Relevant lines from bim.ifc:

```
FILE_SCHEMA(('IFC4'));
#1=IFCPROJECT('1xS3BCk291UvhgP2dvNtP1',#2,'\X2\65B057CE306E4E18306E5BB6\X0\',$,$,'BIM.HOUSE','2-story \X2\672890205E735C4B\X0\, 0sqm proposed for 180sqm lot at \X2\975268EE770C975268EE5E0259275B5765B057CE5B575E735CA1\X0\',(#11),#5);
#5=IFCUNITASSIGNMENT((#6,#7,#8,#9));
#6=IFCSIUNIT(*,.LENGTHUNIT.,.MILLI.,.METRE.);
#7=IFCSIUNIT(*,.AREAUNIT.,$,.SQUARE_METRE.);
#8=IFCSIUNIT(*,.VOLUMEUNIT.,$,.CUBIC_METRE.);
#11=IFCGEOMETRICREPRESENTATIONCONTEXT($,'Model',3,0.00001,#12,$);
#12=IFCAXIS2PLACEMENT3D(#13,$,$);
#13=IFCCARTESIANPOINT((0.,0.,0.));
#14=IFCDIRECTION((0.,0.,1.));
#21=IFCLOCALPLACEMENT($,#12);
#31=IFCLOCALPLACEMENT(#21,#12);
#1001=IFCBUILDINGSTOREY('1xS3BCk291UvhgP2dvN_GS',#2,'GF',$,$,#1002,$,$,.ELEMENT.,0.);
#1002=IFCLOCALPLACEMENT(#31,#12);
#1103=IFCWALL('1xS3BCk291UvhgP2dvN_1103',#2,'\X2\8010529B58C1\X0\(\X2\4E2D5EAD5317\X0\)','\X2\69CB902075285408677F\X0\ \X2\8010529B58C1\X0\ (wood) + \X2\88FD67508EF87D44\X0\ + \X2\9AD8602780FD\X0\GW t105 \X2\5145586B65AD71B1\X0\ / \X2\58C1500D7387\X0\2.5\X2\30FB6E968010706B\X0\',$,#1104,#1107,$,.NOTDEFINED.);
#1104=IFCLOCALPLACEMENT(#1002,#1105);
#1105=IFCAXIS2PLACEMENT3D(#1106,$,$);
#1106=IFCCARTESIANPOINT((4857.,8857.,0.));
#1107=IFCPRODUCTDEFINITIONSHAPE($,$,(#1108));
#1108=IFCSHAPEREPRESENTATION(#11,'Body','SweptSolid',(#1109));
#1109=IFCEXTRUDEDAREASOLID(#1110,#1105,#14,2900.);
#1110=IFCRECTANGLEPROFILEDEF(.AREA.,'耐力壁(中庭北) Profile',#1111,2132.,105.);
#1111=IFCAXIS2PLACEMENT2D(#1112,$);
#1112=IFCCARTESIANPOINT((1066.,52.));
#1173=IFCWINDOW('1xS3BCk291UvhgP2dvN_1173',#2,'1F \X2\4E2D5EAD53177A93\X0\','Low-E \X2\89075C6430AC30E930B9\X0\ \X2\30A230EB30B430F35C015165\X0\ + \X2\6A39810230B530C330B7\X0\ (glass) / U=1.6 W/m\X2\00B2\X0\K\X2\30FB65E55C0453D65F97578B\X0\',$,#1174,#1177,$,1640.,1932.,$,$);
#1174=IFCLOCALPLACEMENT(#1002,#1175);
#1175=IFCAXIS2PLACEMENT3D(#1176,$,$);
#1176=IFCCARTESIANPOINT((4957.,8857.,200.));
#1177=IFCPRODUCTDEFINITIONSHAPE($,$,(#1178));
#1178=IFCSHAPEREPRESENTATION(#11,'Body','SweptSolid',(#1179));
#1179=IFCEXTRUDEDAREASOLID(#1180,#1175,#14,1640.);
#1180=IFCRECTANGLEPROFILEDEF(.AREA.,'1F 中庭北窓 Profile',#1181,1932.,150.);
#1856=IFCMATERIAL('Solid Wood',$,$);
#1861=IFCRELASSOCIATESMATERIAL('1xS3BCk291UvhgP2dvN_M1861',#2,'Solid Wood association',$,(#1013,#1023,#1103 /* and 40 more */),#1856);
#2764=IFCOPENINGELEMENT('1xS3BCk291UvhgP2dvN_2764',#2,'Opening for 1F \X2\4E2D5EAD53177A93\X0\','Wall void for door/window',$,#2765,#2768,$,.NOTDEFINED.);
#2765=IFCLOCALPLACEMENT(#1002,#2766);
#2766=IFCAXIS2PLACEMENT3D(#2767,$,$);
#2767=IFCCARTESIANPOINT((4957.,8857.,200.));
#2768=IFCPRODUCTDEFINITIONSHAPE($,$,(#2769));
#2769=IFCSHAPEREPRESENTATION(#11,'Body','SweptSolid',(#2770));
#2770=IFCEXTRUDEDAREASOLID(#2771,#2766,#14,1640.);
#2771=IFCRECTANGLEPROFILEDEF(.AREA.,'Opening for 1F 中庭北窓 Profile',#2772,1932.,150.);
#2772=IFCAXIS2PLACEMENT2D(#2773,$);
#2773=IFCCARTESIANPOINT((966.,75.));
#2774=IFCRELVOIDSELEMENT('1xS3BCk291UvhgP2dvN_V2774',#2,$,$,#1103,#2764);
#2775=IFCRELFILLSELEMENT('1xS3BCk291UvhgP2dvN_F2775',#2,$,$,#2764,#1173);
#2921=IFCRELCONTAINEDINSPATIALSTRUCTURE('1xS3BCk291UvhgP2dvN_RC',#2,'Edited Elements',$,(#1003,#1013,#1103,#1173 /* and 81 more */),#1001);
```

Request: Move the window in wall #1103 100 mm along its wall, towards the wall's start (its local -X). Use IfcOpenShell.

```python
import ifcopenshell
import ifcopenshell.api.geometry
import ifcopenshell.util.placement

model = ifcopenshell.open("bim.ifc")

window = model.by_id(1173)
opening = window.FillsVoids[0].RelatingOpeningElement
wall = opening.VoidsElements[0].RelatingBuildingElement

wall_matrix = ifcopenshell.util.placement.get_local_placement(wall.ObjectPlacement)
shift = wall_matrix[:3, 0] * -100.0
before = ifcopenshell.util.placement.get_local_placement(window.ObjectPlacement)[:3, 3].copy()

# The window is not placed relative to its opening, so move both.
for product in (opening, window):
    matrix = ifcopenshell.util.placement.get_local_placement(product.ObjectPlacement)
    matrix[:3, 3] += shift
    ifcopenshell.api.geometry.edit_object_placement(model, product=product, matrix=matrix, is_si=False)

after = ifcopenshell.util.placement.get_local_placement(window.ObjectPlacement)[:3, 3]
print("window moved by", (after - before).round(3) + 0.0)

model.write("bim_edited.ifc")
```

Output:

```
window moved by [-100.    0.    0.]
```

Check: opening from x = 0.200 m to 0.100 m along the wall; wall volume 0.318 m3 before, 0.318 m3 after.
